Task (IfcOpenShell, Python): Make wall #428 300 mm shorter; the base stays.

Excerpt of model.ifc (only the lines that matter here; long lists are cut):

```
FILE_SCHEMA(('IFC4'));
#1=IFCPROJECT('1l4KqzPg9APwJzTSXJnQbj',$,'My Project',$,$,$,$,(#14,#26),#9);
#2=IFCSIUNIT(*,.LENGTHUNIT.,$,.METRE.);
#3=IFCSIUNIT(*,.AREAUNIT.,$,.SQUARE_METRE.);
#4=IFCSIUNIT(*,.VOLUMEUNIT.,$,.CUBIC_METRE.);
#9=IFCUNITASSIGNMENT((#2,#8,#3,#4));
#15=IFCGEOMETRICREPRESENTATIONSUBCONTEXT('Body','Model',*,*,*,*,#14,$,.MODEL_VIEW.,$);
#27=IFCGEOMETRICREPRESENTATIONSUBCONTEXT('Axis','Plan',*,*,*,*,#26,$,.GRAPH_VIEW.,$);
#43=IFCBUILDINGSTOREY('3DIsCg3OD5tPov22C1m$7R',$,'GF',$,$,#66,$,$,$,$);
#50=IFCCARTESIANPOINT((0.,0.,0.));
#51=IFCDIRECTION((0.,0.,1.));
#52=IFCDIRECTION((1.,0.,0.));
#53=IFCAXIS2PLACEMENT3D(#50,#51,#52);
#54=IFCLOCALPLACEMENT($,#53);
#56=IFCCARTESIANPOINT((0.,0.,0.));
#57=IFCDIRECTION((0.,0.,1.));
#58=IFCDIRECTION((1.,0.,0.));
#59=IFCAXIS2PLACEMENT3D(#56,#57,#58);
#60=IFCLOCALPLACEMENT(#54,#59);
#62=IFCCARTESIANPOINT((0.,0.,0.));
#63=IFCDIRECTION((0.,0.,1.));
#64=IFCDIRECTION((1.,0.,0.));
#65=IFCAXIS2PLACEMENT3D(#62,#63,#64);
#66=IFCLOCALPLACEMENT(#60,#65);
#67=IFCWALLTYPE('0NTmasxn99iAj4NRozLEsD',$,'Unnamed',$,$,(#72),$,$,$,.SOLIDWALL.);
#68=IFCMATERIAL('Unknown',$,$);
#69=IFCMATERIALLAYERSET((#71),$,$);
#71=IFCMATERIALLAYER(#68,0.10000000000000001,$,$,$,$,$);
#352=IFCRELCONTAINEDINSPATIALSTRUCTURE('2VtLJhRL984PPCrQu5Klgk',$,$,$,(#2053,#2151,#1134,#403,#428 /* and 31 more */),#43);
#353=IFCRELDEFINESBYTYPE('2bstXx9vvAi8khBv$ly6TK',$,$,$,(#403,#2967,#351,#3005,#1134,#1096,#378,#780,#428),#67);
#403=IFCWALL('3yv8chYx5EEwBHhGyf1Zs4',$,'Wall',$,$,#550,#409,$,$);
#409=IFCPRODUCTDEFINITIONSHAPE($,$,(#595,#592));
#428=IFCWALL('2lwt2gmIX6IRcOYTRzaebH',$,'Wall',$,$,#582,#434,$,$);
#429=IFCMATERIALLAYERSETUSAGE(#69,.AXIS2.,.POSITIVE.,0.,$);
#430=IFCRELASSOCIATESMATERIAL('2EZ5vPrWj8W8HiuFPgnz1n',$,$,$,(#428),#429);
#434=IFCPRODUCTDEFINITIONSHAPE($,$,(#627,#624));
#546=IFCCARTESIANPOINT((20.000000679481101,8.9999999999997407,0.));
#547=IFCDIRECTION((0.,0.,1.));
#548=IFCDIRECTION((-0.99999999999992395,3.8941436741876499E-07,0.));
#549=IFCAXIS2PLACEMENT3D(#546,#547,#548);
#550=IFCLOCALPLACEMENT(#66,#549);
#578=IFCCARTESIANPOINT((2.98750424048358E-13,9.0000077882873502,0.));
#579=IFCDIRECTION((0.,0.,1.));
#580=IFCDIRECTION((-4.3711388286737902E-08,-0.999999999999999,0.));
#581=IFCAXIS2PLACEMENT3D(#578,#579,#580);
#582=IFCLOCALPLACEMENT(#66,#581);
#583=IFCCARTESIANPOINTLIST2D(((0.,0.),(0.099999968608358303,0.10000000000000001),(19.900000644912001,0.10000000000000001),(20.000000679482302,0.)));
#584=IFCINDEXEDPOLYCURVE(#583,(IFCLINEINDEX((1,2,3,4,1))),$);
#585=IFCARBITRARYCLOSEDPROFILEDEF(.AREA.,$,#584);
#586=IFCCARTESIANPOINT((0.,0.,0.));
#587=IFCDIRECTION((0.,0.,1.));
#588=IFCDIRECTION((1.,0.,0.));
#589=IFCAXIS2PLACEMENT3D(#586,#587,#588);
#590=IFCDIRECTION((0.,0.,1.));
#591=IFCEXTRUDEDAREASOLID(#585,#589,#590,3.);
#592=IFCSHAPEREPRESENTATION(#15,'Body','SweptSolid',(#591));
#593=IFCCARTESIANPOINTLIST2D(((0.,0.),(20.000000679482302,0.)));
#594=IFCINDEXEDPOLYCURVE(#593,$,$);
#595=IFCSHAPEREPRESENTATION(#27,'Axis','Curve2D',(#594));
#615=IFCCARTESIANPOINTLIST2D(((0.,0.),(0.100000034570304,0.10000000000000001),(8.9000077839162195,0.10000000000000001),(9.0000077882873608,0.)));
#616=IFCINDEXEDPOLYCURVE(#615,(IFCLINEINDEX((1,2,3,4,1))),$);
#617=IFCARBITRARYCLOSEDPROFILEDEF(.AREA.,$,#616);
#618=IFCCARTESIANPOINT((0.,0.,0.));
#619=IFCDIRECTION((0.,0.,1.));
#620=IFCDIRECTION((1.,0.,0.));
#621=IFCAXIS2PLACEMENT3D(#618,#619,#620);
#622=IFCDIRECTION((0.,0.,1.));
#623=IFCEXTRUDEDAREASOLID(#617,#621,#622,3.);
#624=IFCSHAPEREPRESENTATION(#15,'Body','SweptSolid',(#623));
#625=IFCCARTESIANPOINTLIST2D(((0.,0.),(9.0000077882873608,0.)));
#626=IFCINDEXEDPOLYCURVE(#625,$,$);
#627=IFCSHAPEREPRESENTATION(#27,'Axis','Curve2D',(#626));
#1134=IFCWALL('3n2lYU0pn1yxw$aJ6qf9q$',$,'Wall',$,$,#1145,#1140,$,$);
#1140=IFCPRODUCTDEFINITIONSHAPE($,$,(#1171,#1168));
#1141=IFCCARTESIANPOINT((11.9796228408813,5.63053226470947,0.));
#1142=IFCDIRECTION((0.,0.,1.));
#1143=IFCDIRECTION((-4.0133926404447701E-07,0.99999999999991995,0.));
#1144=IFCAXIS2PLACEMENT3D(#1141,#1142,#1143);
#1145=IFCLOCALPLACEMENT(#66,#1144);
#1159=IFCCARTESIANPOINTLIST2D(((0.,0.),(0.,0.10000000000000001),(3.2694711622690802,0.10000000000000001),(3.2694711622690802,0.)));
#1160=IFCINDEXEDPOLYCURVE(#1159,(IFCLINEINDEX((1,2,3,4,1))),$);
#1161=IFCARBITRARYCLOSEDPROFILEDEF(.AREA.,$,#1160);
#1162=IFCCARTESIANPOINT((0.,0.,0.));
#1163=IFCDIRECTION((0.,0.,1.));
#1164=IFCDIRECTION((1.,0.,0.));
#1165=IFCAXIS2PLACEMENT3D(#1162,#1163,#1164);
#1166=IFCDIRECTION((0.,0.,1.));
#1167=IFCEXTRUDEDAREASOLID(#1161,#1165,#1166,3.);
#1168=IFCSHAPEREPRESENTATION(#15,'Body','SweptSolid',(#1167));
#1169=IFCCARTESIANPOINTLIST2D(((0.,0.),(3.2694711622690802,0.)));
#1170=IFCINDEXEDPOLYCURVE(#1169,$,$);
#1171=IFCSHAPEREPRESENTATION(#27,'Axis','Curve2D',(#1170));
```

```python
import ifcopenshell
import ifcopenshell.geom
import ifcopenshell.util.representation
import ifcopenshell.util.shape
import ifcopenshell.util.unit

model = ifcopenshell.open("model.ifc")
unit_scale = ifcopenshell.util.unit.calculate_unit_scale(model)
settings = ifcopenshell.geom.settings()


def volume(element):
    """Net volume in cubic metres, openings subtracted."""
    shape = ifcopenshell.geom.create_shape(settings, element)
    return ifcopenshell.util.shape.get_volume(shape.geometry)


wall = model.by_guid("2lwt2gmIX6IRcOYTRzaebH")
before = volume(wall)

body = ifcopenshell.util.representation.get_representation(wall, "Model", "Body")
solid = body.Items[0]
old_height = solid.Depth
solid.Depth -= 0.3 / unit_scale
after = volume(wall)

print(f"height {old_height:g} -> {solid.Depth:g}, volume {before:.3f} -> {after:.3f} m3")

model.write("model_edited.ifc")
```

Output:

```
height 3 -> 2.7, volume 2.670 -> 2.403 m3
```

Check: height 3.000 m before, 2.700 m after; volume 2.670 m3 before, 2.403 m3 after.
